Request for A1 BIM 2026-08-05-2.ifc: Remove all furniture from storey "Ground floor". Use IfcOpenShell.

First a look at what the model holds.

```python
import ifcopenshell
import ifcopenshell.util.element

model = ifcopenshell.open("A1 BIM 2026-08-05-2.ifc")
print(model.schema)
storey = next(s for s in model.by_type("IfcBuildingStorey") if s.Name == "Ground floor")
furniture = [e for e in ifcopenshell.util.element.get_decomposition(storey) if e.is_a("IfcFurnishingElement")]
seen = {}
for e in furniture:
    element_type = ifcopenshell.util.element.get_type(e)
    name = element_type.Name if element_type not in (None, e) else None
    seen[name] = seen.get(name, 0) + 1
for name, count in sorted(seen.items(), key=str):
    print(count, "x", name)
```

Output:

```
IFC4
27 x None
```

```python
import ifcopenshell
import ifcopenshell.api.root
import ifcopenshell.util.element

model = ifcopenshell.open("A1 BIM 2026-08-05-2.ifc")

storey = next(s for s in model.by_type("IfcBuildingStorey") if s.Name == "Ground floor")
furniture = [e for e in ifcopenshell.util.element.get_decomposition(storey) if e.is_a("IfcFurnishingElement")]

for e in furniture:
    ifcopenshell.api.root.remove_product(model, product=e)
print(len(furniture), "removed")

model.write("A1 BIM 2026-08-05-2_updated.ifc")
```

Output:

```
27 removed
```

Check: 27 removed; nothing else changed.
